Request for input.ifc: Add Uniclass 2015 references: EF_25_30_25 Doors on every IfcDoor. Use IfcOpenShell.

First a look at what the model holds.

```python
import ifcopenshell

model = ifcopenshell.open("input.ifc")
print(model.schema)
print("classifications:", [c.Name for c in model.by_type("IfcClassification")])
for ifc_class in ("IfcDoor", "IfcRoof", "IfcStair", "IfcWall", "IfcWindow"):
    print(ifc_class, len(model.by_type(ifc_class)))
```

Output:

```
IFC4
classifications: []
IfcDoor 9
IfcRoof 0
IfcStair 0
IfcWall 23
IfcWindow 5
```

```python
import ifcopenshell
import ifcopenshell.api.classification

model = ifcopenshell.open("input.ifc")

system = ifcopenshell.api.classification.add_classification(model, classification="Uniclass 2015")

codes = {
    "IfcDoor": ("EF_25_30_25", "Doors"),
}
for ifc_class, (code, name) in codes.items():
    products = model.by_type(ifc_class)
    ifcopenshell.api.classification.add_reference(
        model, products=products, classification=system, identification=code, name=name
    )
    print(code, len(products))

model.write("input_edited.ifc")
```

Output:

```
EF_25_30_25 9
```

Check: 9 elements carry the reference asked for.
